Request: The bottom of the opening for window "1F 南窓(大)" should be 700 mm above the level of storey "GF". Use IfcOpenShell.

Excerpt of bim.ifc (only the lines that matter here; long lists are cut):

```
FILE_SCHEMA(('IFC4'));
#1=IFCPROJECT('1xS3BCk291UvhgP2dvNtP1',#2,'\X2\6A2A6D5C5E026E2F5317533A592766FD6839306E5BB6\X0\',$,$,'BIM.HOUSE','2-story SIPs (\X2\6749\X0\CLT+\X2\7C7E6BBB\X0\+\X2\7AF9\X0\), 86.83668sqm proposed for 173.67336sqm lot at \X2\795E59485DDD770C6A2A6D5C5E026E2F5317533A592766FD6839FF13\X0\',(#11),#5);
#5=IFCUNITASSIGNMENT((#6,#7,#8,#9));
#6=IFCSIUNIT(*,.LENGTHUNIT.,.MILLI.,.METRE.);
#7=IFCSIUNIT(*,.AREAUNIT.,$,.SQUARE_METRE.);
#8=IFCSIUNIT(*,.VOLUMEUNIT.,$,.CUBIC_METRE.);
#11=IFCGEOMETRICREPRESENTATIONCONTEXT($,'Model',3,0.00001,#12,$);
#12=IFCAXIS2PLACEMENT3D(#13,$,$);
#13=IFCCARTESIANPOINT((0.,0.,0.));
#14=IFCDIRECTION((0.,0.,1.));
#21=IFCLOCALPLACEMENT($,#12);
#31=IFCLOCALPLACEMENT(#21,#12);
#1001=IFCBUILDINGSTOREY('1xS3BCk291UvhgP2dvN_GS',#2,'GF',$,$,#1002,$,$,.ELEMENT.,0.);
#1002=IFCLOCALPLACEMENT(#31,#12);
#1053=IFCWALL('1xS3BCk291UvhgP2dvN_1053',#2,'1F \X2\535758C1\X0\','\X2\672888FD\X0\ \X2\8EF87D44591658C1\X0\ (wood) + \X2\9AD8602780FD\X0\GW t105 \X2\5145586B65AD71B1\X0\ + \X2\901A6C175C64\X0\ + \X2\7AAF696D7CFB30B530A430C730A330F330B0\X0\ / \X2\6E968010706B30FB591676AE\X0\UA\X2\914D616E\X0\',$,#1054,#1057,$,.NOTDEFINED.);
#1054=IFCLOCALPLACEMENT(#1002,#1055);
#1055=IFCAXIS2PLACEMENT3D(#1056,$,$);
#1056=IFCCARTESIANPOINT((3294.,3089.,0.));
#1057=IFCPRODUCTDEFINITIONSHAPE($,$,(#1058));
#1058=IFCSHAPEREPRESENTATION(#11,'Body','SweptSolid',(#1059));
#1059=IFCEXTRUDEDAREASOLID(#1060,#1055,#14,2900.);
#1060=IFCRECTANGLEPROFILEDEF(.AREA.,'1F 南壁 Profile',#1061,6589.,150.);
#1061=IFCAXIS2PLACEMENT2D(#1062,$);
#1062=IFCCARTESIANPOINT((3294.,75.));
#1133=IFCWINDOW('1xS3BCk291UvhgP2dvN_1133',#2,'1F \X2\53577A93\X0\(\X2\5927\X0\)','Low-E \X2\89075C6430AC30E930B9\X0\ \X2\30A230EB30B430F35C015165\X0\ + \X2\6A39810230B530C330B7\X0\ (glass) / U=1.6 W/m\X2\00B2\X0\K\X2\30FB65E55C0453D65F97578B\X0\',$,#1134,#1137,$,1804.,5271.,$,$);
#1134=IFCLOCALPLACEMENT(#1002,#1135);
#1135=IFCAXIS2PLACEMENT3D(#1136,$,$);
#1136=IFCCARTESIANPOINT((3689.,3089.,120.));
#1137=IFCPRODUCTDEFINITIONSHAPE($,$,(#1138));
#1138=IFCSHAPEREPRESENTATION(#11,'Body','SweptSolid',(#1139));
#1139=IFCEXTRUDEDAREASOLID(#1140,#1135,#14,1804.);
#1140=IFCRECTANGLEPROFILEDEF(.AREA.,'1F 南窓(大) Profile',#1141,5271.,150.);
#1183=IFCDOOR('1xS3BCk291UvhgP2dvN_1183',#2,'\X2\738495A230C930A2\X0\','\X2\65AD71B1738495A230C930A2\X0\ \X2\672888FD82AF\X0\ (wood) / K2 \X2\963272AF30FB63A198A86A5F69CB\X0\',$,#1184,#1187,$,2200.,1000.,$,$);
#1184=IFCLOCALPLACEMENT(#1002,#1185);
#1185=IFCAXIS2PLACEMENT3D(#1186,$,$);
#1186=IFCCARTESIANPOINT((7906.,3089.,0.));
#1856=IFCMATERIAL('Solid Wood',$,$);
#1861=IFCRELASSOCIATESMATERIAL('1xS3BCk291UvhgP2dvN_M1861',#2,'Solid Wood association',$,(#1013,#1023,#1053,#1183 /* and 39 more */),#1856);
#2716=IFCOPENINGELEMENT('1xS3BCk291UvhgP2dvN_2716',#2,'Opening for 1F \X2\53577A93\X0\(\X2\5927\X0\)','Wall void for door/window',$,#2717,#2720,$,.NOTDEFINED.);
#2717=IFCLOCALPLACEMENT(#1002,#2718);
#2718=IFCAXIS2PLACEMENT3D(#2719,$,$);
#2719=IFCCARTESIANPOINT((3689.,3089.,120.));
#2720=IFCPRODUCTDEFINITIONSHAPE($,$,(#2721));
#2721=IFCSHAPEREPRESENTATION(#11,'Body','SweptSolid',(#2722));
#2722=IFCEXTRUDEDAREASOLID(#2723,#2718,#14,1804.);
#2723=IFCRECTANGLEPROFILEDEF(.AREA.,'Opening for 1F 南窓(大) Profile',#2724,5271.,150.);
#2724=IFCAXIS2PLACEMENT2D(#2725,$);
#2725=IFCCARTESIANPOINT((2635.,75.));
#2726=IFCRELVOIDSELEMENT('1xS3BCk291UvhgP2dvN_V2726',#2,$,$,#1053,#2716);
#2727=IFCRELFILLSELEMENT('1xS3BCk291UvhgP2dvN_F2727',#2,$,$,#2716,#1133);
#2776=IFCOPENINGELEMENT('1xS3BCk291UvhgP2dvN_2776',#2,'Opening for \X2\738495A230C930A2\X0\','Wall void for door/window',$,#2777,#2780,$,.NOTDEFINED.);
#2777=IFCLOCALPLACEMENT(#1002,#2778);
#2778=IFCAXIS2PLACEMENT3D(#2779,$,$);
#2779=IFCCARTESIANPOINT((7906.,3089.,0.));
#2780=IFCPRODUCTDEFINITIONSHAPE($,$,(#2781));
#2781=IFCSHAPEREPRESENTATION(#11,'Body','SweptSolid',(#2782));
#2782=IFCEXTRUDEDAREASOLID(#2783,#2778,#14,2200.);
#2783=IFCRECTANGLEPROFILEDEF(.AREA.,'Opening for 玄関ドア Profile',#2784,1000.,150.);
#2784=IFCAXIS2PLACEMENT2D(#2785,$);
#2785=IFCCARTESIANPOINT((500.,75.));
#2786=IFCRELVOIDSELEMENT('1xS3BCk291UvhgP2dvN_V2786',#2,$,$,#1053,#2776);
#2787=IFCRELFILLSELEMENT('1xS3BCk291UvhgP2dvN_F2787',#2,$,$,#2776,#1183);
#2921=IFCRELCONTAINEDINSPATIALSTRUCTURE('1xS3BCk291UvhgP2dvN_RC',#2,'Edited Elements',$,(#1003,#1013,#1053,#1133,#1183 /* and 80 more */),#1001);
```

```python
import numpy as np
import ifcopenshell
import ifcopenshell.api.geometry
import ifcopenshell.geom
import ifcopenshell.util.element
import ifcopenshell.util.placement
import ifcopenshell.util.shape
import ifcopenshell.util.unit

model = ifcopenshell.open("bim.ifc")
unit_scale = ifcopenshell.util.unit.calculate_unit_scale(model)

window = model.by_id(1133)
opening = window.FillsVoids[0].RelatingOpeningElement
storey = ifcopenshell.util.element.get_container(window, ifc_class="IfcBuildingStorey")
level = ifcopenshell.util.placement.get_local_placement(storey.ObjectPlacement)[2, 3]

# The opening's origin need not be at the sill, so measure its lowest point.
shape = ifcopenshell.geom.create_shape(ifcopenshell.geom.settings(), opening)
bottom = ifcopenshell.util.shape.get_shape_bottom_elevation(shape, shape.geometry) / unit_scale
dz = level + 0.7 / unit_scale - bottom

shift = np.array([0.0, 0.0, dz])
# The window is not placed relative to its opening, so move both.
for product in (opening, window):
    matrix = ifcopenshell.util.placement.get_local_placement(product.ObjectPlacement)
    matrix[:3, 3] += shift
    ifcopenshell.api.geometry.edit_object_placement(model, product=product, matrix=matrix, is_si=False)

print(f"moved by {dz * unit_scale:+.3f} m")

model.write("bim_v2.ifc")
```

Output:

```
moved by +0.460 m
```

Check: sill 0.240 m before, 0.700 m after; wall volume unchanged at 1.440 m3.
